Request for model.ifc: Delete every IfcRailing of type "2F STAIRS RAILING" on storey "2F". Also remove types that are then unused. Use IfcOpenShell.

First a look at what the model holds.

```python
import ifcopenshell
import ifcopenshell.util.element

model = ifcopenshell.open("model.ifc")
print(model.schema)
storey = next(s for s in model.by_type("IfcBuildingStorey") if s.Name == "2F")
railings = [e for e in ifcopenshell.util.element.get_decomposition(storey) if e.is_a("IfcRailing")]
seen = {}
for e in railings:
    element_type = ifcopenshell.util.element.get_type(e)
    name = element_type.Name if element_type not in (None, e) else None
    seen[name] = seen.get(name, 0) + 1
for name, count in sorted(seen.items(), key=str):
    print(count, "x", name)
```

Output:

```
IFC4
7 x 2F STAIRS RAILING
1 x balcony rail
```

```python
import ifcopenshell
import ifcopenshell.api.root
import ifcopenshell.util.element

model = ifcopenshell.open("model.ifc")

storey = next(s for s in model.by_type("IfcBuildingStorey") if s.Name == "2F")
railings = [e for e in ifcopenshell.util.element.get_decomposition(storey) if e.is_a("IfcRailing")]
targets = [e for e in railings if (t := ifcopenshell.util.element.get_type(e)) not in (None, e) and t.Name == "2F STAIRS RAILING"]
types = {ifcopenshell.util.element.get_type(e) for e in targets} - {None, *targets}

for e in targets:
    ifcopenshell.api.root.remove_product(model, product=e)
print(len(targets), "removed")

unused = [t for t in types if not ifcopenshell.util.element.get_types(t)]
for t in unused:
    ifcopenshell.api.root.remove_product(model, product=t)
print(len(unused), "unused types removed")

model.write("model_updated.ifc")
```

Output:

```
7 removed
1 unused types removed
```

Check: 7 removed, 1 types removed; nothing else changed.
